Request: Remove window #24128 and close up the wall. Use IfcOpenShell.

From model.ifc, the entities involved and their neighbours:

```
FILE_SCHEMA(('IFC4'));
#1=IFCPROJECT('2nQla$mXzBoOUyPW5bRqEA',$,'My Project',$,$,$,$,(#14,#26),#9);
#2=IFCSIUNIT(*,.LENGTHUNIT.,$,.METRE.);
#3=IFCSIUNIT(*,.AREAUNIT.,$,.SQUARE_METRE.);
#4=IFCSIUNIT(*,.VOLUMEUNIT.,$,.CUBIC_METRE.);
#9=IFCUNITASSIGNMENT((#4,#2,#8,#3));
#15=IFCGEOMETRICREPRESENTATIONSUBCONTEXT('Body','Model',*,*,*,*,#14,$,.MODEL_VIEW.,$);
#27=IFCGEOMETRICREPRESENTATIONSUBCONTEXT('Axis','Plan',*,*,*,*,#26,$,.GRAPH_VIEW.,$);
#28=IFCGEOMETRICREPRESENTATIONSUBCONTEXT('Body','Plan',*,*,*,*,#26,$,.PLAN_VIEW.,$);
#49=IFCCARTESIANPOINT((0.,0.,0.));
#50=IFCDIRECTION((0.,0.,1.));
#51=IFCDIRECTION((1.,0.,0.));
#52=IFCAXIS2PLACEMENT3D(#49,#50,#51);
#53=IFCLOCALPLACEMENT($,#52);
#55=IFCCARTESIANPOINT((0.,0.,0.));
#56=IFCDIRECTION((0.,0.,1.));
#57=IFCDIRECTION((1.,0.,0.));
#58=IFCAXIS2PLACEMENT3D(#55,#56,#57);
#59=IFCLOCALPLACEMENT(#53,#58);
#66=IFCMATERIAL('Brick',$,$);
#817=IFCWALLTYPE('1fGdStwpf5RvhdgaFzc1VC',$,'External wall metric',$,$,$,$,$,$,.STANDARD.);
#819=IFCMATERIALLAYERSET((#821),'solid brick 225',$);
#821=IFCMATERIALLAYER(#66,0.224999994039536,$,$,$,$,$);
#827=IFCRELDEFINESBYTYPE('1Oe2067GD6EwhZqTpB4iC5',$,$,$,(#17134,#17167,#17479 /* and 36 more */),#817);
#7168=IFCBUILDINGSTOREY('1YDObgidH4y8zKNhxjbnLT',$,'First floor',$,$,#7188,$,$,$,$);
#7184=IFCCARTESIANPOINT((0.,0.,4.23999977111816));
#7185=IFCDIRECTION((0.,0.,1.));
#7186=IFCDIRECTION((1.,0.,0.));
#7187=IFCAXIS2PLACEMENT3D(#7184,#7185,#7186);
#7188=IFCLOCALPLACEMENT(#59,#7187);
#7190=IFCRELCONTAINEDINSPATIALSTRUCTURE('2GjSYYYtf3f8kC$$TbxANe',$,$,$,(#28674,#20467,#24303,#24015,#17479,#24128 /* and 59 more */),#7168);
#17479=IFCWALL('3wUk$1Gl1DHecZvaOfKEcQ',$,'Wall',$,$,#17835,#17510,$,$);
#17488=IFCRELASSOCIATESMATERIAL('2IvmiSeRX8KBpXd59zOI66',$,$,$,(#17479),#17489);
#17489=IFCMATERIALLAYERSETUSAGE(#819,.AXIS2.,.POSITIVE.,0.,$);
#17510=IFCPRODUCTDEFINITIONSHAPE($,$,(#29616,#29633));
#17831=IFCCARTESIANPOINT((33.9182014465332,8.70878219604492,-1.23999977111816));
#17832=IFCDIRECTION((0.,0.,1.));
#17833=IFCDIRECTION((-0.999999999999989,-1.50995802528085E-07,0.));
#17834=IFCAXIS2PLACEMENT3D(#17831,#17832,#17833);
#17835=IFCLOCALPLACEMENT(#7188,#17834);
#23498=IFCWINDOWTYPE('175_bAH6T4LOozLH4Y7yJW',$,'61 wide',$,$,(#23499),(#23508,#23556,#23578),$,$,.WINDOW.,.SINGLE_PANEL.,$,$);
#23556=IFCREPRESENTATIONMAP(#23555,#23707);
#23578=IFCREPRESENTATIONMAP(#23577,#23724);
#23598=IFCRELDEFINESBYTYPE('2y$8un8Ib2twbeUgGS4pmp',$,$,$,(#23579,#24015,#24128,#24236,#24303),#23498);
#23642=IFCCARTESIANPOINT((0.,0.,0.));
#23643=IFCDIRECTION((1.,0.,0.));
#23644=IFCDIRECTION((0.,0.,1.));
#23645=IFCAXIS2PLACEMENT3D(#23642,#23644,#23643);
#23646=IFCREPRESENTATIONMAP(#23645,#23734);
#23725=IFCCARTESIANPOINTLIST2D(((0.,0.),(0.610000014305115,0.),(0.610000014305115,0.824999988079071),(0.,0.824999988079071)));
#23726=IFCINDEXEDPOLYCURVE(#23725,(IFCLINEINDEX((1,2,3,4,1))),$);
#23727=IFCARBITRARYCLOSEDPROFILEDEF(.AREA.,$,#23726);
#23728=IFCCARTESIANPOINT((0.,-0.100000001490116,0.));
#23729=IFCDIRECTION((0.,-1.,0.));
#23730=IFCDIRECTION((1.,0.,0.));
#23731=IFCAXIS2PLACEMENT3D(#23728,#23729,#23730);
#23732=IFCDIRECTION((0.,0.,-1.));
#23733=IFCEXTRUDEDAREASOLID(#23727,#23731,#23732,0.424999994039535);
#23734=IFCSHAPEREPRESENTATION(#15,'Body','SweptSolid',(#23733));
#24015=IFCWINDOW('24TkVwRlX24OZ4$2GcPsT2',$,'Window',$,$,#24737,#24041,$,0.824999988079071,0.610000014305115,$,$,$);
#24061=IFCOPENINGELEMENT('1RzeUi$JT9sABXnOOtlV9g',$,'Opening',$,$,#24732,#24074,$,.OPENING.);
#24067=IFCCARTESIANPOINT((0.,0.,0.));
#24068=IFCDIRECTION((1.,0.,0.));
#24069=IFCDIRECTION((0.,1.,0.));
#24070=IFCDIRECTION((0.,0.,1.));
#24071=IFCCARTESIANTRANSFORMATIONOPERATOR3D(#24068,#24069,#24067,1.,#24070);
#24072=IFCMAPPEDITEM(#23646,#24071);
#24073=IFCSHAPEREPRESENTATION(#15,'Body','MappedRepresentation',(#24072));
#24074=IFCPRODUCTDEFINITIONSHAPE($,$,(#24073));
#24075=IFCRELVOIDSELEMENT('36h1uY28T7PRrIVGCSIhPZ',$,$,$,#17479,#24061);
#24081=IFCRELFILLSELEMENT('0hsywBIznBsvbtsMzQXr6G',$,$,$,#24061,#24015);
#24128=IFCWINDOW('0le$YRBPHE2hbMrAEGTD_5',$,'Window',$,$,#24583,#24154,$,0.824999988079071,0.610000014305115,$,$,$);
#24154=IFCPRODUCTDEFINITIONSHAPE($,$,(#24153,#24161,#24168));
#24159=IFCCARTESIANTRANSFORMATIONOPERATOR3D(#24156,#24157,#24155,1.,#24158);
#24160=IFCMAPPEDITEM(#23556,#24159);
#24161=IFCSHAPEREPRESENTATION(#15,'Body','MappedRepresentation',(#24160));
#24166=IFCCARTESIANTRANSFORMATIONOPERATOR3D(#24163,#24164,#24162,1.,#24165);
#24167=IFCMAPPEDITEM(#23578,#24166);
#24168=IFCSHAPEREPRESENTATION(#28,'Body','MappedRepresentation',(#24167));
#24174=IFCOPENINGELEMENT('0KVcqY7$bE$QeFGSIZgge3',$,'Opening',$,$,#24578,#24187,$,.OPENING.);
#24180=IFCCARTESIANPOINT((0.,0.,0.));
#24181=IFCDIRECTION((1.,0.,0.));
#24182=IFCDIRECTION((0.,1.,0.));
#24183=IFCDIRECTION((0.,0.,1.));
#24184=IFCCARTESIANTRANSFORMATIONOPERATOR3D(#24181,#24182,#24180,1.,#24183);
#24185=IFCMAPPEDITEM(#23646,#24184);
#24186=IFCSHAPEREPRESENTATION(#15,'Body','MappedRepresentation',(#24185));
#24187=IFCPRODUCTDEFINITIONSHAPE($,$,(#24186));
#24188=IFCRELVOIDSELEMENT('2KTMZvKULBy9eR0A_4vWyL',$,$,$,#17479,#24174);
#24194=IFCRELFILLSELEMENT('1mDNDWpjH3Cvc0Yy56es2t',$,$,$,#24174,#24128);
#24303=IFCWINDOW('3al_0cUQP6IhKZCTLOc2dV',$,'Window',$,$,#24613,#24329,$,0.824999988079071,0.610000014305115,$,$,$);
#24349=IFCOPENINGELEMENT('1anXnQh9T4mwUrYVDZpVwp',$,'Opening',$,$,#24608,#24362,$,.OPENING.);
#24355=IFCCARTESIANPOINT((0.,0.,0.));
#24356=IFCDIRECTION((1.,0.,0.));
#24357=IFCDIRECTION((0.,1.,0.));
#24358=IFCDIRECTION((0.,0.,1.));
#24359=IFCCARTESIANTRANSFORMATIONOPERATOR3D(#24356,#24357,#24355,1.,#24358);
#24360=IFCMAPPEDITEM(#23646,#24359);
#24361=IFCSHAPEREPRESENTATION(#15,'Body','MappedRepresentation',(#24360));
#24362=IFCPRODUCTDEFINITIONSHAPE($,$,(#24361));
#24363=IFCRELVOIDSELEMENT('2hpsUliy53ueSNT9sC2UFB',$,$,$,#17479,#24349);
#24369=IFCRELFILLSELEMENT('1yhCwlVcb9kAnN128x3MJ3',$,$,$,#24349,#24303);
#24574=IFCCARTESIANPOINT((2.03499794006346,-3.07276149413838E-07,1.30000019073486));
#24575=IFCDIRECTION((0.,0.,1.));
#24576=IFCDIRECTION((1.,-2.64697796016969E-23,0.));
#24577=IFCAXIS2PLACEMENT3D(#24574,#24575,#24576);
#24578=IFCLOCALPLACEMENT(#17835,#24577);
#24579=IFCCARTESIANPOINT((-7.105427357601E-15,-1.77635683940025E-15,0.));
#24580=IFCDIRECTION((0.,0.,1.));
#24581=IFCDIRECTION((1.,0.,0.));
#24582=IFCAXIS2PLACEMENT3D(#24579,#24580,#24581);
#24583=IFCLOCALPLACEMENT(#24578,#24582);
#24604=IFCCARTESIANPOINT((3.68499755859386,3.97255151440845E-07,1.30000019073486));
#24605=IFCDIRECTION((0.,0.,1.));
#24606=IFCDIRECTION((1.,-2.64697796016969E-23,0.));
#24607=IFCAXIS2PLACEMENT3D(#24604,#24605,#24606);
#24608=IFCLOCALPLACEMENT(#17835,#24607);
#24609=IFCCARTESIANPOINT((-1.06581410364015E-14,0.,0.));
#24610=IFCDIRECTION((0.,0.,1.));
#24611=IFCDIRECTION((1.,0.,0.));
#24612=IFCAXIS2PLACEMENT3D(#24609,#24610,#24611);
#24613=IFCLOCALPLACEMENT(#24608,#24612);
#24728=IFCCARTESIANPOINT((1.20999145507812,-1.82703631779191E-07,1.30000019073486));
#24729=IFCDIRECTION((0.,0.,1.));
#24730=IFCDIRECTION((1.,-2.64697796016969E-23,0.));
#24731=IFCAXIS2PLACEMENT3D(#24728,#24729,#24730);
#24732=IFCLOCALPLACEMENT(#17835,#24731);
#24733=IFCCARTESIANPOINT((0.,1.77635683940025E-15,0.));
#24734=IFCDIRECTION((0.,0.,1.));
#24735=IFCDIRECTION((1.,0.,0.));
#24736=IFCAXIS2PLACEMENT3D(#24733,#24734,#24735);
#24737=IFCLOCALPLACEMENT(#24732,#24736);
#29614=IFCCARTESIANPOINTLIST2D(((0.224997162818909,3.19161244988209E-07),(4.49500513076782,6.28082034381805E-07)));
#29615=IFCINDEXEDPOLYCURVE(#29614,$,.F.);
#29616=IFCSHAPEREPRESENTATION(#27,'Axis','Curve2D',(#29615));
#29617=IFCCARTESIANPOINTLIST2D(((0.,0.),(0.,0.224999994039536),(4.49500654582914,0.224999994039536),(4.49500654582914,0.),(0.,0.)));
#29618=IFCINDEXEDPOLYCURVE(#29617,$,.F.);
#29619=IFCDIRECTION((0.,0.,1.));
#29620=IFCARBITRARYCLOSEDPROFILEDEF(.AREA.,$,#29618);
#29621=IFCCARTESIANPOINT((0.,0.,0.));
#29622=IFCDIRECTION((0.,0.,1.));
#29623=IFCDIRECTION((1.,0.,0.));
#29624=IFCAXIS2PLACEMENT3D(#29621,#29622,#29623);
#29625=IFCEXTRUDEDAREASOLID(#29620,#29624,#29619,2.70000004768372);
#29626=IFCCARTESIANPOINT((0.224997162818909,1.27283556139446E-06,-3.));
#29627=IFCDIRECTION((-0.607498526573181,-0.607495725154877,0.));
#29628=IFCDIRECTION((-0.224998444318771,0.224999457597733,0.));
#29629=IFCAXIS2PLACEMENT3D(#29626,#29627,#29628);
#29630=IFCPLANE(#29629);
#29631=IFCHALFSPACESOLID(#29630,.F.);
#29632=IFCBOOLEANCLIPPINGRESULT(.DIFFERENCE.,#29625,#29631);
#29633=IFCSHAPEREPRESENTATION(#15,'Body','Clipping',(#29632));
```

```python
import ifcopenshell
import ifcopenshell.api.feature
import ifcopenshell.api.root
import ifcopenshell.geom
import ifcopenshell.util.shape

model = ifcopenshell.open("model.ifc")
settings = ifcopenshell.geom.settings()


def volume(element):
    """Net volume in cubic metres, openings subtracted."""
    shape = ifcopenshell.geom.create_shape(settings, element)
    return ifcopenshell.util.shape.get_volume(shape.geometry)


window = model.by_guid("0le$YRBPHE2hbMrAEGTD_5")
opening = window.FillsVoids[0].RelatingOpeningElement
wall = opening.VoidsElements[0].RelatingBuildingElement
before = volume(wall)

ifcopenshell.api.root.remove_product(model, product=window)
ifcopenshell.api.feature.remove_feature(model, feature=opening)

after = volume(wall)

print(f"wall volume {before:.3f} -> {after:.3f} m3")

model.write("model-out.ifc")
```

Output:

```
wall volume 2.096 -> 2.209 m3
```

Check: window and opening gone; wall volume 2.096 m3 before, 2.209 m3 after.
